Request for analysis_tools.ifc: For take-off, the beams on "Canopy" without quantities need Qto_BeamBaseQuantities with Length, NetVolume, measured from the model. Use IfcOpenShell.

First a look at what the model holds.

```python
import ifcopenshell
import ifcopenshell.util.element
import ifcopenshell.util.unit

model = ifcopenshell.open("analysis_tools.ifc")
print(model.schema)
for unit_type in ("LENGTHUNIT", "AREAUNIT", "VOLUMEUNIT"):
    print(unit_type, ifcopenshell.util.unit.calculate_unit_scale(model, unit_type))
storey = next(s for s in model.by_type("IfcBuildingStorey") if s.Name == "Canopy")
beams = [e for e in ifcopenshell.util.element.get_decomposition(storey) if e.is_a("IfcBeam")]
for e in sorted(beams, key=lambda e: e.id()):
    print(e.id(), e.is_a(), e.Name, list(ifcopenshell.util.element.get_psets(e, qtos_only=True)), sep=" | ")
```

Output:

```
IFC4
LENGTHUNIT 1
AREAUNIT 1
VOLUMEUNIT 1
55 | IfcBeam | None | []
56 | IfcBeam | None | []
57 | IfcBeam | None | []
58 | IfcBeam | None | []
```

```python
import ifcopenshell
import ifcopenshell.api.pset
import ifcopenshell.geom
import ifcopenshell.util.element
import ifcopenshell.util.shape
import ifcopenshell.util.unit

model = ifcopenshell.open("analysis_tools.ifc")
unit_scale = ifcopenshell.util.unit.calculate_unit_scale(model)
volume_scale = ifcopenshell.util.unit.calculate_unit_scale(model, "VOLUMEUNIT")
settings = ifcopenshell.geom.settings()

storey = next(s for s in model.by_type("IfcBuildingStorey") if s.Name == "Canopy")
beams = [e for e in ifcopenshell.util.element.get_decomposition(storey) if e.is_a("IfcBeam")]

for e in sorted(beams, key=lambda e: e.id()):
    if ifcopenshell.util.element.get_psets(e, qtos_only=True, should_inherit=False):
        continue
    # Geometry comes back in metres, in the element's own axes.
    shape = ifcopenshell.geom.create_shape(settings, e)
    values = {
        "Length": ifcopenshell.util.shape.get_max_xyz(shape.geometry) / unit_scale,
        "NetVolume": ifcopenshell.util.shape.get_volume(shape.geometry) / volume_scale,
    }
    qto = ifcopenshell.api.pset.add_qto(model, product=e, name="Qto_BeamBaseQuantities")
    ifcopenshell.api.pset.edit_qto(model, qto=qto, properties=values)
    print(e.id(), {k: round(v, 3) for k, v in values.items()})

model.write("analysis_tools-out.ifc")
```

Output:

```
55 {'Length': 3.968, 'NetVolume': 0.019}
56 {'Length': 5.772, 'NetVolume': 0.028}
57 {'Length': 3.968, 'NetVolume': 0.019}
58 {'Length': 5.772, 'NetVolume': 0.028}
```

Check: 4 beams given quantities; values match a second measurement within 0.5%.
